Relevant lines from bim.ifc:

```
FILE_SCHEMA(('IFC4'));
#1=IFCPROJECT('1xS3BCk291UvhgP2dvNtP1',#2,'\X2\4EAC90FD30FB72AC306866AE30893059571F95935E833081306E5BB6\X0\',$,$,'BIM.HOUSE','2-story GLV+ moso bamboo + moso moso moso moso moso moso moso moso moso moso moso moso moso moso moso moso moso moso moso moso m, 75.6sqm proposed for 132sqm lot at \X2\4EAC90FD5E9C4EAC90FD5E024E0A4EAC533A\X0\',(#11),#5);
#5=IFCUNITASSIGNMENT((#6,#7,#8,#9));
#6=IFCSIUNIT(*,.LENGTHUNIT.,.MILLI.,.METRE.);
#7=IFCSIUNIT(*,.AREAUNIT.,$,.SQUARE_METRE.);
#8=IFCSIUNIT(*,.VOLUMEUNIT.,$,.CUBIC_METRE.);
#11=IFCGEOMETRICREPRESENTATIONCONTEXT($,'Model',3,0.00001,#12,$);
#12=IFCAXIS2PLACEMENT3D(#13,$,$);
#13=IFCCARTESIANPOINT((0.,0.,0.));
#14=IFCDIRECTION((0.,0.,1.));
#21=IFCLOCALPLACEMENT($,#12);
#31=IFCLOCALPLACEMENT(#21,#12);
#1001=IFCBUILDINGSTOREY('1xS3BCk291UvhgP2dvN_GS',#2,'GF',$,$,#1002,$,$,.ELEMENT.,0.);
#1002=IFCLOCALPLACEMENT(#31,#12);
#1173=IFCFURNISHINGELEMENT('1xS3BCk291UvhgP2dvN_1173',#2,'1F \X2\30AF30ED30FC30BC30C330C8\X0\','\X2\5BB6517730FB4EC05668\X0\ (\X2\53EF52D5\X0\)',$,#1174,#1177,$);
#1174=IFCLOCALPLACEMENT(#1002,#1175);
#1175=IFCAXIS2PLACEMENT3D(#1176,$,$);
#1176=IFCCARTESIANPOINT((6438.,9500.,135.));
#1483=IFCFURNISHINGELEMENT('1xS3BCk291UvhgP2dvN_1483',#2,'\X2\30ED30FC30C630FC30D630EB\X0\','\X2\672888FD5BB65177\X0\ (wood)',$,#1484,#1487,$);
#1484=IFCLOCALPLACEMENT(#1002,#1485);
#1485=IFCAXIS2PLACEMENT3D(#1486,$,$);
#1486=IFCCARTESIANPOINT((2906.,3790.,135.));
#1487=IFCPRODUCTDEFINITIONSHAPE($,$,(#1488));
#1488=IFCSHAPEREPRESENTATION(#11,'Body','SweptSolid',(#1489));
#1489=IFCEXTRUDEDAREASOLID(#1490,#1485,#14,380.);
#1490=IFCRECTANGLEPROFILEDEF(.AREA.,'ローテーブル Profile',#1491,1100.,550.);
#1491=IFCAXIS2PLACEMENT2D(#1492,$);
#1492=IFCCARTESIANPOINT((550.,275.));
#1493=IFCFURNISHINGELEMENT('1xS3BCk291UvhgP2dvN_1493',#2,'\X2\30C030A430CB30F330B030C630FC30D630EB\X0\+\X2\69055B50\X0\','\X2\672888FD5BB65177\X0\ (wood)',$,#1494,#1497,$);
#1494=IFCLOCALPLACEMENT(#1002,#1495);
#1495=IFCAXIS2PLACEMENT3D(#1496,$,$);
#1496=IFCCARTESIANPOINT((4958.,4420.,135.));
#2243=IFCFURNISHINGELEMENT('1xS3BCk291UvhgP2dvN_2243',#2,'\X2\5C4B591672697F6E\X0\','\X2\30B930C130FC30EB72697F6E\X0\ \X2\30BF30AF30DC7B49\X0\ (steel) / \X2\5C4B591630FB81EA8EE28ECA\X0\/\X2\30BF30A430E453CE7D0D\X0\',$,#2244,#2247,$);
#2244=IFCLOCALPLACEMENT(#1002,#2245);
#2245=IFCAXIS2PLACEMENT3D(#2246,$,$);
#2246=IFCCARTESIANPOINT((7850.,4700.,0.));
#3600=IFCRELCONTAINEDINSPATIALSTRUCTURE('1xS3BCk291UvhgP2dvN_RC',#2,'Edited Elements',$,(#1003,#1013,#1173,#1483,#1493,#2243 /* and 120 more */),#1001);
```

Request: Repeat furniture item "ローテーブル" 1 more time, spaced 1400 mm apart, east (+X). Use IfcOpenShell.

```python
import numpy as np
import ifcopenshell
import ifcopenshell.api.geometry
import ifcopenshell.api.root
import ifcopenshell.util.element
import ifcopenshell.util.placement

model = ifcopenshell.open("bim.ifc")


def reuse_history(source, copy):
    """copy_class also copies each property set's owner history, people and application; keep the originals."""
    for rel in copy.IsDefinedBy:
        if rel.is_a("IfcRelDefinesByProperties") and (history := rel.RelatingPropertyDefinition.OwnerHistory):
            rel.RelatingPropertyDefinition.OwnerHistory = source.OwnerHistory
            ifcopenshell.util.element.remove_deep2(model, history)


source = model.by_id(1483)
base = ifcopenshell.util.placement.get_local_placement(source.ObjectPlacement)
step = np.array([1.0, 0.0, 0.0]) * 1400.0

for i in range(1, 2):
    copy = ifcopenshell.api.root.copy_class(model, product=source)
    copy.Representation = ifcopenshell.util.element.copy_deep(
        model, source.Representation, exclude=["IfcGeometricRepresentationContext", "IfcRepresentationMap"]
    )
    reuse_history(source, copy)
    matrix = base.copy()
    matrix[:3, 3] += i * step
    print("added at", matrix[:3, 3].round(3) + 0.0)
    ifcopenshell.api.geometry.edit_object_placement(model, product=copy, matrix=matrix, is_si=False)

model.write("bim_v2.ifc")
```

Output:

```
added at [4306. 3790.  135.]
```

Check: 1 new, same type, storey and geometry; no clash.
